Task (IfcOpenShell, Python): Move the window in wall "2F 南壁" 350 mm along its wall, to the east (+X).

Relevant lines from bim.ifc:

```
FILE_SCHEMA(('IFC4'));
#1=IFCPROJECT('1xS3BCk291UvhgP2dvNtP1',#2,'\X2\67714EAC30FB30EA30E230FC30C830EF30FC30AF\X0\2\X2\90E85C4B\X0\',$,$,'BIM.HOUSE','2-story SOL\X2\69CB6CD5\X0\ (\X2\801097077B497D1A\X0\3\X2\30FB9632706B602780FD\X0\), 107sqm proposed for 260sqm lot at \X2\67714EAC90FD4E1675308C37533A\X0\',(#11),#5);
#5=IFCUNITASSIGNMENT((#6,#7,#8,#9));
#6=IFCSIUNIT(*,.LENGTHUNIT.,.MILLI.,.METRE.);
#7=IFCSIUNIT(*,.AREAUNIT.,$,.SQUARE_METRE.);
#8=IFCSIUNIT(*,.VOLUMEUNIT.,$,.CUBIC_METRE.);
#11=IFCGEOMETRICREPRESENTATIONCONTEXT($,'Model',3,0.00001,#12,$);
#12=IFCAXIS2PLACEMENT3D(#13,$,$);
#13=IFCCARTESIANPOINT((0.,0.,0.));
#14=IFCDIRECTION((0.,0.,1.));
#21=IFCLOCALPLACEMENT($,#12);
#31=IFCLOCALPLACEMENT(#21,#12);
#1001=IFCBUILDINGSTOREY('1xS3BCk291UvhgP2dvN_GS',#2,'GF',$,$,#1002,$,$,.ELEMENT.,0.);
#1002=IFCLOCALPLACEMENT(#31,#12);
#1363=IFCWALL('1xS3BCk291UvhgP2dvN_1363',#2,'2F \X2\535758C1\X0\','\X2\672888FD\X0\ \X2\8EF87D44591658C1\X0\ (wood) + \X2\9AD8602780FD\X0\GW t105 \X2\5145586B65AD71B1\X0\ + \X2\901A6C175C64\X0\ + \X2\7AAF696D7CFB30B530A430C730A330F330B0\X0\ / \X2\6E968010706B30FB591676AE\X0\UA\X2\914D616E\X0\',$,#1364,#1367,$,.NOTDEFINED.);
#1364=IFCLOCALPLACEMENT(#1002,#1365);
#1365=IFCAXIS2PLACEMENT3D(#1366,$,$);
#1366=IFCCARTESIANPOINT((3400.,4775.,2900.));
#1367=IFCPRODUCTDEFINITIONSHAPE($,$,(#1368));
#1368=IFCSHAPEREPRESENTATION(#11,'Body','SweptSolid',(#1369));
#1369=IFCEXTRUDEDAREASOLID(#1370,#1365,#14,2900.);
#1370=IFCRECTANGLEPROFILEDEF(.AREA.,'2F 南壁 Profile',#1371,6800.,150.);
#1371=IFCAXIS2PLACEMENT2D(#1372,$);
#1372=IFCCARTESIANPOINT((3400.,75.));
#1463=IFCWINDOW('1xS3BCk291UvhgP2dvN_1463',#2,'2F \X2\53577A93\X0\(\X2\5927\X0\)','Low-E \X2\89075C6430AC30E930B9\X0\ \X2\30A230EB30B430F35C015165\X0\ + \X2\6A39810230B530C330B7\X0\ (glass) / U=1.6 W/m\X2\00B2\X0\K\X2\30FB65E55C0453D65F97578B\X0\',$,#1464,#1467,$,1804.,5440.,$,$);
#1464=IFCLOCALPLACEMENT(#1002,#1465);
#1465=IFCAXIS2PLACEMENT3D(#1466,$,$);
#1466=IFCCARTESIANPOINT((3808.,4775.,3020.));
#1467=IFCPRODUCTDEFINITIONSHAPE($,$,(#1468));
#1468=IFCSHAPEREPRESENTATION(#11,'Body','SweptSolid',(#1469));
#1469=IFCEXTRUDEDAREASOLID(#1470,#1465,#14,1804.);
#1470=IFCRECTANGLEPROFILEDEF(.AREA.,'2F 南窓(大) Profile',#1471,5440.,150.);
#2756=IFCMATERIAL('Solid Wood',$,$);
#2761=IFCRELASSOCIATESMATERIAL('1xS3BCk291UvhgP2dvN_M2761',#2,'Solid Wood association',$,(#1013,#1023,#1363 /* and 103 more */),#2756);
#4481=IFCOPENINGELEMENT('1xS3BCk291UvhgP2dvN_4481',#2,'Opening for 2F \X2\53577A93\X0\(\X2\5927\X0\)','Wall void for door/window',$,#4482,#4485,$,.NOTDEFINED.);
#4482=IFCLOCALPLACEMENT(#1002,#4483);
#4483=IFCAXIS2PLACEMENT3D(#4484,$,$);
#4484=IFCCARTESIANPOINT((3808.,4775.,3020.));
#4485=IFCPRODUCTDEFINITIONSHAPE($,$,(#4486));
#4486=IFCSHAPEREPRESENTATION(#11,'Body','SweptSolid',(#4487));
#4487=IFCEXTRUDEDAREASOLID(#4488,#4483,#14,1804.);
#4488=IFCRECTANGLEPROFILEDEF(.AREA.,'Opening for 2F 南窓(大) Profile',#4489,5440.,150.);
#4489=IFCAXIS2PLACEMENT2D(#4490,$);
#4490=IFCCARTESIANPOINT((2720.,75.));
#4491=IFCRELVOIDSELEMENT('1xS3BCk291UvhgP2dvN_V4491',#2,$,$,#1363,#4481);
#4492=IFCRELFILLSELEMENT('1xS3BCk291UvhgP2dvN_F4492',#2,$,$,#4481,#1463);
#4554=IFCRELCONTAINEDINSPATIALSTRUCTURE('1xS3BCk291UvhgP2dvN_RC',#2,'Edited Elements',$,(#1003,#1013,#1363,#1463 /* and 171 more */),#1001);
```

```python
import ifcopenshell
import ifcopenshell.api.geometry
import ifcopenshell.util.placement

model = ifcopenshell.open("bim.ifc")

window = model.by_guid("1xS3BCk291UvhgP2dvN_1463")
opening = window.FillsVoids[0].RelatingOpeningElement
wall = opening.VoidsElements[0].RelatingBuildingElement

wall_matrix = ifcopenshell.util.placement.get_local_placement(wall.ObjectPlacement)
shift = wall_matrix[:3, 0] * 350.0
before = ifcopenshell.util.placement.get_local_placement(window.ObjectPlacement)[:3, 3].copy()

# The window is not placed relative to its opening, so move both.
for product in (opening, window):
    matrix = ifcopenshell.util.placement.get_local_placement(product.ObjectPlacement)
    matrix[:3, 3] += shift
    ifcopenshell.api.geometry.edit_object_placement(model, product=product, matrix=matrix, is_si=False)

after = ifcopenshell.util.placement.get_local_placement(window.ObjectPlacement)[:3, 3]
print("window moved by", (after - before).round(3) + 0.0)

model.write("bim_v2.ifc")
```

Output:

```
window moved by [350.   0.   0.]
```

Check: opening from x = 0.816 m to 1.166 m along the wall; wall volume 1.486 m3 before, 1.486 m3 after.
